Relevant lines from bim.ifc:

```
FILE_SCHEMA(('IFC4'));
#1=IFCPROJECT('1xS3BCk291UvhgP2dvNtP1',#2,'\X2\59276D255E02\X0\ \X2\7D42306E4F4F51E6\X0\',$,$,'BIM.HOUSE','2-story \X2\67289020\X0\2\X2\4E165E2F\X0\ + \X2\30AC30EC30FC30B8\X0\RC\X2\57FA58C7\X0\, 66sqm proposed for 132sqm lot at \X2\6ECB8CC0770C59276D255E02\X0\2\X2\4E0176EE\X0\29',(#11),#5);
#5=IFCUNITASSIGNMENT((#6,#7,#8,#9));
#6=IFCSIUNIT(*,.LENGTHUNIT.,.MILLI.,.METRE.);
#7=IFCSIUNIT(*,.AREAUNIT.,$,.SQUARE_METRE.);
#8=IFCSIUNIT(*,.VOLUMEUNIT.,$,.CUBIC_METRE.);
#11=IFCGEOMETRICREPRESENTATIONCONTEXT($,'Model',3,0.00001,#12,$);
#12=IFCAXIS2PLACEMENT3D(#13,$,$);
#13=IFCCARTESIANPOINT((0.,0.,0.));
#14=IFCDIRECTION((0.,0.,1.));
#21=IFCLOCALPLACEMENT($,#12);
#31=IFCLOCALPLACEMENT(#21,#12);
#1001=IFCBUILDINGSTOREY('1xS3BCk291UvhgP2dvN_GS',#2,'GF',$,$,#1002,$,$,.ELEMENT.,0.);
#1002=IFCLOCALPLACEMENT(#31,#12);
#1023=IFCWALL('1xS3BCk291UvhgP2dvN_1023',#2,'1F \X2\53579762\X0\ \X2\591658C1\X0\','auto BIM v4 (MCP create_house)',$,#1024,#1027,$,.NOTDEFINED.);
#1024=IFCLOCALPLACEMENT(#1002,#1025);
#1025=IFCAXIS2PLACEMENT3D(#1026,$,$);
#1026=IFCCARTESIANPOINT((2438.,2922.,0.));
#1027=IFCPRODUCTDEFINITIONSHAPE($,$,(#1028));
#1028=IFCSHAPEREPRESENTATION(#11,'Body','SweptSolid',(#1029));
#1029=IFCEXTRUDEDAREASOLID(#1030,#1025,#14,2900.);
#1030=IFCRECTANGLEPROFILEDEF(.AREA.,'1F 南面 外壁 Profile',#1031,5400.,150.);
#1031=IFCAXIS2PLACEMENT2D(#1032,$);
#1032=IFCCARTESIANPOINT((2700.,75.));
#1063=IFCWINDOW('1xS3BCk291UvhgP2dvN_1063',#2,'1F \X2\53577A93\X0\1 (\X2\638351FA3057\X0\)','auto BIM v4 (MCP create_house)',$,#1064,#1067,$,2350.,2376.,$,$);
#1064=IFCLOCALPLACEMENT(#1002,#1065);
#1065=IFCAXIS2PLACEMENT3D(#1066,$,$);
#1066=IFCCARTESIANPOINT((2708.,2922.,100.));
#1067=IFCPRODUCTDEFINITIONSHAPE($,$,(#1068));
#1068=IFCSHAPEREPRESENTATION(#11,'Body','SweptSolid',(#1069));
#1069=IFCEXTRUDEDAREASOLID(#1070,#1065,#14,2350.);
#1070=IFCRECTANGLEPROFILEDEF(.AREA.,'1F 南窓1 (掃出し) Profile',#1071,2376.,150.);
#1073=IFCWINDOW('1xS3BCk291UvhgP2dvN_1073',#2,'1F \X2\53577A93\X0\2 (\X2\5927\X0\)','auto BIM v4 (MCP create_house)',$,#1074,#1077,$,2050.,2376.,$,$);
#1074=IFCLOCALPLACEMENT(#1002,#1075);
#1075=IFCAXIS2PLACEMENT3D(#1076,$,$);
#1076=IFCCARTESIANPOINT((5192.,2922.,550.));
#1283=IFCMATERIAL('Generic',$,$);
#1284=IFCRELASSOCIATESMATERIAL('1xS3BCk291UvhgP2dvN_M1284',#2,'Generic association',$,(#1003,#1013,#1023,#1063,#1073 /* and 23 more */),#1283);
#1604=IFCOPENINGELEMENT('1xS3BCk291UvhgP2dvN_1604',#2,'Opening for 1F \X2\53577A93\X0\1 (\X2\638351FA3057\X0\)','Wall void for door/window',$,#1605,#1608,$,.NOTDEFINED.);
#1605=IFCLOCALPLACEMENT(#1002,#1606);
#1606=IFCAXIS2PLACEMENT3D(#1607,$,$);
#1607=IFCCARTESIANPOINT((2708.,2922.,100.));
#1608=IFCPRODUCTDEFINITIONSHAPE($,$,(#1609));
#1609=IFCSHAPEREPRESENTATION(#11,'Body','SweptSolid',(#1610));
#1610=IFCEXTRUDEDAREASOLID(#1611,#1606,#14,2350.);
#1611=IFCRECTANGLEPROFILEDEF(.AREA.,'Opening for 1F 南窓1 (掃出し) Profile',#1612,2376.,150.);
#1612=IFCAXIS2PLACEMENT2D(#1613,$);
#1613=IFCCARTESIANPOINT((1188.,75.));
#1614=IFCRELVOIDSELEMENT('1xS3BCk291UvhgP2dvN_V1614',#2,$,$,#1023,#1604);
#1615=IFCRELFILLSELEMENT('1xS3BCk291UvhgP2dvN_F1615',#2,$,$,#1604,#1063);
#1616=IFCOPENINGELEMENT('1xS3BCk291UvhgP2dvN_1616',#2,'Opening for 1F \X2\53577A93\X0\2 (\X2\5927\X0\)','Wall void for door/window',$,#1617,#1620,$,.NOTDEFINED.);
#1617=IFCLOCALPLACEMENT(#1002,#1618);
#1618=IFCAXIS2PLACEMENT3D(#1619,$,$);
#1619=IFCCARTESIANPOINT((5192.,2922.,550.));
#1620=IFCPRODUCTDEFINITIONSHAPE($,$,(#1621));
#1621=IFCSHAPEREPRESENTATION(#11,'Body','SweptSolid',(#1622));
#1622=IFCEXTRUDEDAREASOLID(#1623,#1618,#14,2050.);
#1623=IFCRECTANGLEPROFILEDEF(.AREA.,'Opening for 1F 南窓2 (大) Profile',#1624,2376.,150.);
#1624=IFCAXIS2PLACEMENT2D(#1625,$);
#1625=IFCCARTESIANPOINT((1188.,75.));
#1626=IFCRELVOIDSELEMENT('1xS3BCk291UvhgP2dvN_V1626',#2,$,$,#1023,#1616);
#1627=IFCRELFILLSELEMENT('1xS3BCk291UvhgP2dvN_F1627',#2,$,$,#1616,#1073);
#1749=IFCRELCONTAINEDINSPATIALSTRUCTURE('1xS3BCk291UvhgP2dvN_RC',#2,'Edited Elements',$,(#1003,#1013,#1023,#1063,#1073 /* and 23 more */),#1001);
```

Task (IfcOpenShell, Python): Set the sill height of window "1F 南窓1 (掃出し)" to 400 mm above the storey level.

```python
import numpy as np
import ifcopenshell
import ifcopenshell.api.geometry
import ifcopenshell.geom
import ifcopenshell.util.element
import ifcopenshell.util.placement
import ifcopenshell.util.shape
import ifcopenshell.util.unit

model = ifcopenshell.open("bim.ifc")
unit_scale = ifcopenshell.util.unit.calculate_unit_scale(model)

window = model.by_guid("1xS3BCk291UvhgP2dvN_1063")
opening = window.FillsVoids[0].RelatingOpeningElement
storey = ifcopenshell.util.element.get_container(window, ifc_class="IfcBuildingStorey")
level = ifcopenshell.util.placement.get_local_placement(storey.ObjectPlacement)[2, 3]

# The opening's origin need not be at the sill, so measure its lowest point.
shape = ifcopenshell.geom.create_shape(ifcopenshell.geom.settings(), opening)
bottom = ifcopenshell.util.shape.get_shape_bottom_elevation(shape, shape.geometry) / unit_scale
dz = level + 0.4 / unit_scale - bottom

shift = np.array([0.0, 0.0, dz])
# The window is not placed relative to its opening, so move both.
for product in (opening, window):
    matrix = ifcopenshell.util.placement.get_local_placement(product.ObjectPlacement)
    matrix[:3, 3] += shift
    ifcopenshell.api.geometry.edit_object_placement(model, product=product, matrix=matrix, is_si=False)

print(f"moved by {dz * unit_scale:+.3f} m")

model.write("bim_updated.ifc")
```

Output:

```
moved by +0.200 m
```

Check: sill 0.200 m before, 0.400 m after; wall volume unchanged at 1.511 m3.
